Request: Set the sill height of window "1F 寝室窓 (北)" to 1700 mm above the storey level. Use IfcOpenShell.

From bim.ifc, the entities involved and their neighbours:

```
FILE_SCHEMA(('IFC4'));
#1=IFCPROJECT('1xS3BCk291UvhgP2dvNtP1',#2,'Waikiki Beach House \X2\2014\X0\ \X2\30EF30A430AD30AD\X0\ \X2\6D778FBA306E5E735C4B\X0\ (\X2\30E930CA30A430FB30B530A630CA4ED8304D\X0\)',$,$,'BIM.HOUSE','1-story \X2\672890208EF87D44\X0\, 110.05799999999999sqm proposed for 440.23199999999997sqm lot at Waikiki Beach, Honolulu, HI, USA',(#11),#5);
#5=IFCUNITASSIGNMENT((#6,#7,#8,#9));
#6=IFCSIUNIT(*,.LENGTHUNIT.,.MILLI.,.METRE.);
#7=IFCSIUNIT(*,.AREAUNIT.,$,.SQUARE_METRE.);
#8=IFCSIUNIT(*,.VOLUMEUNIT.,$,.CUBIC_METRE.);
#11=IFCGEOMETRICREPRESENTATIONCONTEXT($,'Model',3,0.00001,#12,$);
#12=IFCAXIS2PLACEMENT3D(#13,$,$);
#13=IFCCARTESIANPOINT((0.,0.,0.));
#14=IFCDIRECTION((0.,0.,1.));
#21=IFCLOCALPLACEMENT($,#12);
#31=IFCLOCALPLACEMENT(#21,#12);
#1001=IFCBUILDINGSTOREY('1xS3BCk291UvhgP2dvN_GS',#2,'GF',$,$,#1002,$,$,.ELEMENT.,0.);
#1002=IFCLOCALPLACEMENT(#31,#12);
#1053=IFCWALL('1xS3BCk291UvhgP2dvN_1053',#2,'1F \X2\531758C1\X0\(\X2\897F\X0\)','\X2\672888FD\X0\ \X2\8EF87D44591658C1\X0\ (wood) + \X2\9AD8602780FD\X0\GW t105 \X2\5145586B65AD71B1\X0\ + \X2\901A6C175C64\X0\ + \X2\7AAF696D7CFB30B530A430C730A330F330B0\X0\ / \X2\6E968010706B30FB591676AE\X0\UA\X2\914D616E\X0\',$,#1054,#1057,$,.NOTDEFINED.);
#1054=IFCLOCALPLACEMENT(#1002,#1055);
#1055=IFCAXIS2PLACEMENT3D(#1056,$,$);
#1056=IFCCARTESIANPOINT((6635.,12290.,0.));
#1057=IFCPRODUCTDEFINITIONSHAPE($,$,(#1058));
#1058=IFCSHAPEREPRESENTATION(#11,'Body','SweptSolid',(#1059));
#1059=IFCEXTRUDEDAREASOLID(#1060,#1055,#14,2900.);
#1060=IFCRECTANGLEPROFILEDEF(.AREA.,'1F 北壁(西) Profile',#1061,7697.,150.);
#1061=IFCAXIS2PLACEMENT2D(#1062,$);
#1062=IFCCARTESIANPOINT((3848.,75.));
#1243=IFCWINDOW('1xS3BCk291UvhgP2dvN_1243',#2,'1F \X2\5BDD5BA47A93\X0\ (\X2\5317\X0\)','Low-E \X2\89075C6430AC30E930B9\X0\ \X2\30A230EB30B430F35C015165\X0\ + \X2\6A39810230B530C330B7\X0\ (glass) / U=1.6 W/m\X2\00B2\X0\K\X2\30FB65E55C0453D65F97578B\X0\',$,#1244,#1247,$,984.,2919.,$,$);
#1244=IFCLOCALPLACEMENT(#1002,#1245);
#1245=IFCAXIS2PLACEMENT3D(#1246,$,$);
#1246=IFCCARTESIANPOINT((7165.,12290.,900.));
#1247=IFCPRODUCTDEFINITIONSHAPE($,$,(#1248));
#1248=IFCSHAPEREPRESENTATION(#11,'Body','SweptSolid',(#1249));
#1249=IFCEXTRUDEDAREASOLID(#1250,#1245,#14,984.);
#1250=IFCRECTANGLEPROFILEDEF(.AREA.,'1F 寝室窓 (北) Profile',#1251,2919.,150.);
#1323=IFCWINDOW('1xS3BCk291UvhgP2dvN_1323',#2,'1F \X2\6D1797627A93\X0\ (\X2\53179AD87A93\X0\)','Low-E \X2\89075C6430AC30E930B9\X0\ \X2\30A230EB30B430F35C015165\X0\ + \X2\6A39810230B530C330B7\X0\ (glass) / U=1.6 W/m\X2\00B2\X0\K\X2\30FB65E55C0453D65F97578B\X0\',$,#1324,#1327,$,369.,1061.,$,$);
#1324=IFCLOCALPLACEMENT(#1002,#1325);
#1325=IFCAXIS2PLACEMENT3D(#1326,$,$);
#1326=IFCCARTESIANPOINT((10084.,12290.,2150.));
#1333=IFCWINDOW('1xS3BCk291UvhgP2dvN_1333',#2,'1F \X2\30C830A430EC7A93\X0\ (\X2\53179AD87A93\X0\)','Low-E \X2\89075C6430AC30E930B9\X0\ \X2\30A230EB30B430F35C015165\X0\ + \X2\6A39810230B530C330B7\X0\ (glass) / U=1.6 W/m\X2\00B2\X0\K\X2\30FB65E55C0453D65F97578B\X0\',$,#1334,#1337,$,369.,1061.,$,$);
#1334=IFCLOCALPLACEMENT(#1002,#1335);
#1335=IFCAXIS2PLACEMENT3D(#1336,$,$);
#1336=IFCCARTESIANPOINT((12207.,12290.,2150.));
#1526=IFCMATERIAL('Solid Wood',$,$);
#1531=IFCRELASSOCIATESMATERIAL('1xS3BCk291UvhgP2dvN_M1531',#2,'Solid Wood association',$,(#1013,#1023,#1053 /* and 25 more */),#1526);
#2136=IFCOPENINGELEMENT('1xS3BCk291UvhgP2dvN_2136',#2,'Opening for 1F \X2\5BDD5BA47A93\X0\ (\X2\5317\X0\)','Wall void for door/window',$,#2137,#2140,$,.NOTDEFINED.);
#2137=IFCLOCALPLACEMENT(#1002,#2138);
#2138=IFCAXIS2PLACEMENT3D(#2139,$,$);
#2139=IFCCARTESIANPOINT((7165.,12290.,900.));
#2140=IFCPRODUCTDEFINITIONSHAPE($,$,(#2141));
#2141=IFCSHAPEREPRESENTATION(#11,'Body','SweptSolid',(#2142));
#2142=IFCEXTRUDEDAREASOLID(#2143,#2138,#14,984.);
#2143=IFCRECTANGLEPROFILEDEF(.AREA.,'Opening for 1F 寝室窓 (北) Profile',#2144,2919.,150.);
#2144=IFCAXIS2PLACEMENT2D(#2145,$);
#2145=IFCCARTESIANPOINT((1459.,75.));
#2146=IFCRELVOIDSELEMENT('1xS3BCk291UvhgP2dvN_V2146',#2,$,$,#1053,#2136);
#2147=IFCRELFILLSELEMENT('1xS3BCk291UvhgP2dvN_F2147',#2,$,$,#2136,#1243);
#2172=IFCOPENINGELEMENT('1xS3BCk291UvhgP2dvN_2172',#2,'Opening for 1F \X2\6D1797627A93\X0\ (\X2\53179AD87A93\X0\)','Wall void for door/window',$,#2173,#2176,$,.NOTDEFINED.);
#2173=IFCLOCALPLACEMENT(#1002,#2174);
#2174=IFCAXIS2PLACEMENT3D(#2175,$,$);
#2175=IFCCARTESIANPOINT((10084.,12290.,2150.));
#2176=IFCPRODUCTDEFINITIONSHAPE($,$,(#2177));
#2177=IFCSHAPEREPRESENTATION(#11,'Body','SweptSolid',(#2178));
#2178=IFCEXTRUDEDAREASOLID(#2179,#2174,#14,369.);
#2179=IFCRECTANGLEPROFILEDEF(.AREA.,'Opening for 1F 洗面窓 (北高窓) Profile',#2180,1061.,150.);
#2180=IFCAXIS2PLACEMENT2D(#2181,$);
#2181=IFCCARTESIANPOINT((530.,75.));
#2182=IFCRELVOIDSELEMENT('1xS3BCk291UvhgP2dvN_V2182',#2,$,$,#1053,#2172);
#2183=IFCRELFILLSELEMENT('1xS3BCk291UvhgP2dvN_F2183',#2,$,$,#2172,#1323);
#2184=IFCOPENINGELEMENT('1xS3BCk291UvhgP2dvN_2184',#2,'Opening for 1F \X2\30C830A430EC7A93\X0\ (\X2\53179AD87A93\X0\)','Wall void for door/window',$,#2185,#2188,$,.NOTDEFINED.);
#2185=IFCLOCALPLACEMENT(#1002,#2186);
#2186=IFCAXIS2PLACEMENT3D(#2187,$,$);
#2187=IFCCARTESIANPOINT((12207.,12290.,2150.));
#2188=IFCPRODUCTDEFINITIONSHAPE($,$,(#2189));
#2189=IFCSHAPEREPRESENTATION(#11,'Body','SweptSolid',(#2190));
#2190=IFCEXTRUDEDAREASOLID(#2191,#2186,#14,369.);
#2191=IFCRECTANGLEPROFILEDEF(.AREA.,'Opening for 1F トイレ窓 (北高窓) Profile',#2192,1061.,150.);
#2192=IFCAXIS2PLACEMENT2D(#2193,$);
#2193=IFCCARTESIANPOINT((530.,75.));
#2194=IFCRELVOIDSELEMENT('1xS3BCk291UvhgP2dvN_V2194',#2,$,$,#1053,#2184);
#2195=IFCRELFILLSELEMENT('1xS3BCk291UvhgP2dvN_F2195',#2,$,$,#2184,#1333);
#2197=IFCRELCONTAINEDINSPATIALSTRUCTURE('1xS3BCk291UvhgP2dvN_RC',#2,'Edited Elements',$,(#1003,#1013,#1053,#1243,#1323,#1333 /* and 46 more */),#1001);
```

```python
import numpy as np
import ifcopenshell
import ifcopenshell.api.geometry
import ifcopenshell.geom
import ifcopenshell.util.element
import ifcopenshell.util.placement
import ifcopenshell.util.shape
import ifcopenshell.util.unit

model = ifcopenshell.open("bim.ifc")
unit_scale = ifcopenshell.util.unit.calculate_unit_scale(model)

window = model.by_guid("1xS3BCk291UvhgP2dvN_1243")
opening = window.FillsVoids[0].RelatingOpeningElement
storey = ifcopenshell.util.element.get_container(window, ifc_class="IfcBuildingStorey")
level = ifcopenshell.util.placement.get_local_placement(storey.ObjectPlacement)[2, 3]

# The opening's origin need not be at the sill, so measure its lowest point.
shape = ifcopenshell.geom.create_shape(ifcopenshell.geom.settings(), opening)
bottom = ifcopenshell.util.shape.get_shape_bottom_elevation(shape, shape.geometry) / unit_scale
dz = level + 1.7 / unit_scale - bottom

shift = np.array([0.0, 0.0, dz])
# The window is not placed relative to its opening, so move both.
for product in (opening, window):
    matrix = ifcopenshell.util.placement.get_local_placement(product.ObjectPlacement)
    matrix[:3, 3] += shift
    ifcopenshell.api.geometry.edit_object_placement(model, product=product, matrix=matrix, is_si=False)

print(f"moved by {dz * unit_scale:+.3f} m")

model.write("bim_updated.ifc")
```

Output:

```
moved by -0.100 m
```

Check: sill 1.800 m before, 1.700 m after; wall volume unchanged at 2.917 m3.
